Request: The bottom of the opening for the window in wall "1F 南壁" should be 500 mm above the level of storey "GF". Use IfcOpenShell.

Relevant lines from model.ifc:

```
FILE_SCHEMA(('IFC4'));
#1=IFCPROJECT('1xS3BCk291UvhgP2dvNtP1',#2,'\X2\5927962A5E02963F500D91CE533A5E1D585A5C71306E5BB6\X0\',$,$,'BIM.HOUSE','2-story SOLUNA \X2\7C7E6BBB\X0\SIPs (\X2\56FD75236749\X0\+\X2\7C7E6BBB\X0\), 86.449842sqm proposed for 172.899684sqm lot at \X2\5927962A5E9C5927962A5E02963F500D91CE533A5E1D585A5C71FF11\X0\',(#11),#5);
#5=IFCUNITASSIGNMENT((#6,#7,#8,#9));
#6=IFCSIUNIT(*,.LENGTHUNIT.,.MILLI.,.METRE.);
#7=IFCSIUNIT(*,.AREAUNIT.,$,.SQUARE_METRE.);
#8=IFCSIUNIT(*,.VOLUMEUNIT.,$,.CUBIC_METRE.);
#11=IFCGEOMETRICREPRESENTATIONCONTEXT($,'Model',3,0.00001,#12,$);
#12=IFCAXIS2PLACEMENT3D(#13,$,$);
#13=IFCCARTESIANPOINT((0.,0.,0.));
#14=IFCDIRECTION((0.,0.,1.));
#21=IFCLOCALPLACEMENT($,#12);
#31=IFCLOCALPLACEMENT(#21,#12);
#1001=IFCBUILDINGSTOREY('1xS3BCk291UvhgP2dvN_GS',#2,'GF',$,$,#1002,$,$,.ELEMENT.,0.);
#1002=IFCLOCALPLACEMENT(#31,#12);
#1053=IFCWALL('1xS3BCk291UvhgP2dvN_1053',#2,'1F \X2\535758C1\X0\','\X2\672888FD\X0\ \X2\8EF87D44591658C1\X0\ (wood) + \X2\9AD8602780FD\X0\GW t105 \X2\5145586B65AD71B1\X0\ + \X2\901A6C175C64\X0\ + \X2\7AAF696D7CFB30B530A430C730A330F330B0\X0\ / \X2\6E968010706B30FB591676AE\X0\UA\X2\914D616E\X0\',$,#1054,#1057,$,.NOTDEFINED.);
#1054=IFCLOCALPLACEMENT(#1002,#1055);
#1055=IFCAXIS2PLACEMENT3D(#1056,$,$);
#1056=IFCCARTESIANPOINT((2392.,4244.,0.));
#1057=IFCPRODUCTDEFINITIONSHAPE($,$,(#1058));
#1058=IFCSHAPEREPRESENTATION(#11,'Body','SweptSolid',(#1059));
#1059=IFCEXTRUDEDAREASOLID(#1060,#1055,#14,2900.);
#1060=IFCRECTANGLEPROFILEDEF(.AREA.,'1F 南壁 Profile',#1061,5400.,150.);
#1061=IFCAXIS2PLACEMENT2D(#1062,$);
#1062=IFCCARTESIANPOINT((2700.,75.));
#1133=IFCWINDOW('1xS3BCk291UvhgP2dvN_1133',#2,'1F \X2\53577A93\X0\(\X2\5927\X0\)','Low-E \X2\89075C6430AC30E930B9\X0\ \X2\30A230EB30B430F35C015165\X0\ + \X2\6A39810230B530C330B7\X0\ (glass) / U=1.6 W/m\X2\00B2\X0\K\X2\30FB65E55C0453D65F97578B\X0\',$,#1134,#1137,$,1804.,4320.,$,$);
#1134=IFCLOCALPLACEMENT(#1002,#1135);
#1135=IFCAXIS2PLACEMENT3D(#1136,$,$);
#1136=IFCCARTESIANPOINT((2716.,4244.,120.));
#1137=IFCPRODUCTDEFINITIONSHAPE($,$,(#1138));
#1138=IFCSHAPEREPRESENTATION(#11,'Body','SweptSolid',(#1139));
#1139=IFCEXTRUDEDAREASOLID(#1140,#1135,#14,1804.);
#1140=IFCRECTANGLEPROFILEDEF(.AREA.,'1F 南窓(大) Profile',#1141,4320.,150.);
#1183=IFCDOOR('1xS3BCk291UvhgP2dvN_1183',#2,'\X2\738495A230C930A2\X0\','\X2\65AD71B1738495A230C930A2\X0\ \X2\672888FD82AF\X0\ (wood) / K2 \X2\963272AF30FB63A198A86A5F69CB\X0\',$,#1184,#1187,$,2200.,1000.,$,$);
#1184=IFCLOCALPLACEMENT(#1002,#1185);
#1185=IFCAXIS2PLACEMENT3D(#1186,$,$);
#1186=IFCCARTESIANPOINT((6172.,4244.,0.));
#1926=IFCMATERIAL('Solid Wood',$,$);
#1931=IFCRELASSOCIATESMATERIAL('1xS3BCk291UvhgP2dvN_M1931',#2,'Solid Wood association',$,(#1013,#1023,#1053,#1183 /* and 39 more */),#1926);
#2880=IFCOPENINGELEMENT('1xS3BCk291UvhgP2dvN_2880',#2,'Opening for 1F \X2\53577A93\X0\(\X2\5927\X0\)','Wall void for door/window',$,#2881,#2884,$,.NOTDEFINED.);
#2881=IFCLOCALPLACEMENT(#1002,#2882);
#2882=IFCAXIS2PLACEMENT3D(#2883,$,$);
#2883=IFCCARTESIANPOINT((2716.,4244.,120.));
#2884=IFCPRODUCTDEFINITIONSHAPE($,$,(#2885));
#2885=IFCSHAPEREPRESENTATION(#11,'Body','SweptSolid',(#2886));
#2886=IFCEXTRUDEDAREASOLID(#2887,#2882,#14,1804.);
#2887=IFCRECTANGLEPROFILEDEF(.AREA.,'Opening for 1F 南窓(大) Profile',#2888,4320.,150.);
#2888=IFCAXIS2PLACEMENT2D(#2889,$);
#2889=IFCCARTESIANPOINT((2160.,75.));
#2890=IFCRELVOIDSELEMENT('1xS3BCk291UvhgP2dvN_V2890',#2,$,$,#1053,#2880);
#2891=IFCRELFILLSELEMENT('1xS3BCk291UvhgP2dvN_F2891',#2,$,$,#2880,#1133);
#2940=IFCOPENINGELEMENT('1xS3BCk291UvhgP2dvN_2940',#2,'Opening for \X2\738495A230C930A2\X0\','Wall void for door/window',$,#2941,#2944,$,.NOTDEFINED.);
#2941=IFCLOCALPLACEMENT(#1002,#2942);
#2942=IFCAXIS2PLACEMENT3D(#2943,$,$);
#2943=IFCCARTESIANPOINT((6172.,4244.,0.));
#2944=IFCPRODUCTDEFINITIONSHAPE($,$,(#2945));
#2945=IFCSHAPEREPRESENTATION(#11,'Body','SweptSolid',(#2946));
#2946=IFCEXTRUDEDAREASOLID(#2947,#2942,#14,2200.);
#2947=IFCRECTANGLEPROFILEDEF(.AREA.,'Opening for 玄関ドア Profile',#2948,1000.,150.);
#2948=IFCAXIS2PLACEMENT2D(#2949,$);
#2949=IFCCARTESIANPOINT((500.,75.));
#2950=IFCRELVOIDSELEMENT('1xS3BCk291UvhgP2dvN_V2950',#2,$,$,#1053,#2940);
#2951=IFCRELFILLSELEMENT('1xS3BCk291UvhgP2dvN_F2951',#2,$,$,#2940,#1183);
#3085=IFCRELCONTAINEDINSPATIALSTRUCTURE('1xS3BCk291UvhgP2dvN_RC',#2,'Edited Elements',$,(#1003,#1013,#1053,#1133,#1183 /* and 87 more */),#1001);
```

```python
import numpy as np
import ifcopenshell
import ifcopenshell.api.geometry
import ifcopenshell.geom
import ifcopenshell.util.element
import ifcopenshell.util.placement
import ifcopenshell.util.shape
import ifcopenshell.util.unit

model = ifcopenshell.open("model.ifc")
unit_scale = ifcopenshell.util.unit.calculate_unit_scale(model)

window = model.by_id(1133)
opening = window.FillsVoids[0].RelatingOpeningElement
storey = ifcopenshell.util.element.get_container(window, ifc_class="IfcBuildingStorey")
level = ifcopenshell.util.placement.get_local_placement(storey.ObjectPlacement)[2, 3]

# The opening's origin need not be at the sill, so measure its lowest point.
shape = ifcopenshell.geom.create_shape(ifcopenshell.geom.settings(), opening)
bottom = ifcopenshell.util.shape.get_shape_bottom_elevation(shape, shape.geometry) / unit_scale
dz = level + 0.5 / unit_scale - bottom

shift = np.array([0.0, 0.0, dz])
# The window is not placed relative to its opening, so move both.
for product in (opening, window):
    matrix = ifcopenshell.util.placement.get_local_placement(product.ObjectPlacement)
    matrix[:3, 3] += shift
    ifcopenshell.api.geometry.edit_object_placement(model, product=product, matrix=matrix, is_si=False)

print(f"moved by {dz * unit_scale:+.3f} m")

model.write("model_v2.ifc")
```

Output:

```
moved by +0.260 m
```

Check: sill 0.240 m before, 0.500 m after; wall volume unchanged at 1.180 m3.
